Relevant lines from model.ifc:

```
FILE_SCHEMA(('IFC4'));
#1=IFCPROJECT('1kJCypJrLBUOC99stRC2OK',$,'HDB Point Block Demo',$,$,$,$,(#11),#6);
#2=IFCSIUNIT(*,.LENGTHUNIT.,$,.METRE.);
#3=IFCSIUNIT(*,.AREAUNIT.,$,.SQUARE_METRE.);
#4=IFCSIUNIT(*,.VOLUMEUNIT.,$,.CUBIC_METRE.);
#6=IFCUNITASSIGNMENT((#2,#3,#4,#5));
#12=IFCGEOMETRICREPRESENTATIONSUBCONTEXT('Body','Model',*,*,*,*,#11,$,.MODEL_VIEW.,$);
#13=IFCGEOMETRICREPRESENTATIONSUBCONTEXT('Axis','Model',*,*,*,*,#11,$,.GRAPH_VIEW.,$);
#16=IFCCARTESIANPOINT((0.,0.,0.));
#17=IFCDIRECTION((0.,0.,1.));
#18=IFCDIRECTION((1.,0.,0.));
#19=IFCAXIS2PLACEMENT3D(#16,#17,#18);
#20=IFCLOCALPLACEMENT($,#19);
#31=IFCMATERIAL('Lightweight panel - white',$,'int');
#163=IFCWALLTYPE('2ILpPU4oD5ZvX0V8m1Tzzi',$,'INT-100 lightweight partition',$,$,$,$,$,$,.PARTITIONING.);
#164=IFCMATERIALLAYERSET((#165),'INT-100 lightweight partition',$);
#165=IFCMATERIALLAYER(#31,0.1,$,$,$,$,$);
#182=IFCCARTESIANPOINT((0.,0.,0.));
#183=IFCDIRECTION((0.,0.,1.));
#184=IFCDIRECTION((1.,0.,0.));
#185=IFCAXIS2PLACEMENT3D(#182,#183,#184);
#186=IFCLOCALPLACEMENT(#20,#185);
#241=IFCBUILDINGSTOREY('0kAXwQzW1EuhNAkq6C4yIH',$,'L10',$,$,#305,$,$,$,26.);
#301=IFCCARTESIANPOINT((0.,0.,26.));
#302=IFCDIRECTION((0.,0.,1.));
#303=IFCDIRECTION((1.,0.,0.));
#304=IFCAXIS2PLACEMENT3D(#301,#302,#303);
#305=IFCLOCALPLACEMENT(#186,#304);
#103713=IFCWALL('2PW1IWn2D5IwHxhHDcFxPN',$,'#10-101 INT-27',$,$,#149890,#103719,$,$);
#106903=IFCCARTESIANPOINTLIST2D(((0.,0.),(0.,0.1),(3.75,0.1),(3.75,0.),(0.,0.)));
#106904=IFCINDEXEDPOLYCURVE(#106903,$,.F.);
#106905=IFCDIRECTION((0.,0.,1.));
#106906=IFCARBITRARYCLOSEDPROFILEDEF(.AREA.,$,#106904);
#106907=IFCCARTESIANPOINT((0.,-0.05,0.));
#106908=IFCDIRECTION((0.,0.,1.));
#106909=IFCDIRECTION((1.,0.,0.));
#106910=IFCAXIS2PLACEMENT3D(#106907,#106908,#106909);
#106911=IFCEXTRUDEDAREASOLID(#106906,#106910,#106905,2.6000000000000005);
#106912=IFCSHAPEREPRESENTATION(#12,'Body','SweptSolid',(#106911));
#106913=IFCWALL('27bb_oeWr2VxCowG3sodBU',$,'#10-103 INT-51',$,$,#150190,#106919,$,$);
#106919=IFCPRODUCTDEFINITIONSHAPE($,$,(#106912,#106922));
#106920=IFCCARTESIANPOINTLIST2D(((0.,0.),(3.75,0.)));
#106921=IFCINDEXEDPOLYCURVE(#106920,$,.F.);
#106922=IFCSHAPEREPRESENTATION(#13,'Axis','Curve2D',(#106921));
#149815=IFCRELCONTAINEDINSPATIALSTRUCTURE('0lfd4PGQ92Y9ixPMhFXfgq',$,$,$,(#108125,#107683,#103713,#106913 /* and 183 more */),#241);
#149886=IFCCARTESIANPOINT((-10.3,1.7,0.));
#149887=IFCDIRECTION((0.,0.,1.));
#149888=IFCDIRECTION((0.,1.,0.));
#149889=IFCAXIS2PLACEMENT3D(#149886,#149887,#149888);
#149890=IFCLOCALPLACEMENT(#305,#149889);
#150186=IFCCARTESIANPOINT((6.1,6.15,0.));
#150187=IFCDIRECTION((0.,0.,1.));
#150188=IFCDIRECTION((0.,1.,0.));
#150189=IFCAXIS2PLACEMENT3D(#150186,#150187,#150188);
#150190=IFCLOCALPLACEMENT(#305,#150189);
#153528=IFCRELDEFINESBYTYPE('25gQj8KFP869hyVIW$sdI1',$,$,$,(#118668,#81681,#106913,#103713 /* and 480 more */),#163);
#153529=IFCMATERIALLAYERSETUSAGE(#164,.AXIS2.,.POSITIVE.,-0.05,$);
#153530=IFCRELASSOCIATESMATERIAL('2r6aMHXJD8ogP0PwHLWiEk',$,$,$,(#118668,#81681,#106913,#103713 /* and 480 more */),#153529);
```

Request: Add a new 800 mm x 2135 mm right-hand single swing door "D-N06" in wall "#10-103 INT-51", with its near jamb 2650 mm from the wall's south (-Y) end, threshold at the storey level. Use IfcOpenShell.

```python
import numpy as np
import ifcopenshell
import ifcopenshell.api.feature
import ifcopenshell.api.geometry
import ifcopenshell.api.root
import ifcopenshell.api.spatial
import ifcopenshell.geom
import ifcopenshell.util.element
import ifcopenshell.util.placement
import ifcopenshell.util.representation
import ifcopenshell.util.shape
import ifcopenshell.util.unit

model = ifcopenshell.open("model.ifc")
unit_scale = ifcopenshell.util.unit.calculate_unit_scale(model)
settings = ifcopenshell.geom.settings()


def volume(element):
    """Net volume in cubic metres, openings subtracted."""
    shape = ifcopenshell.geom.create_shape(settings, element)
    return ifcopenshell.util.shape.get_volume(shape.geometry)


wall = model.by_id(106913)
storey = ifcopenshell.util.element.get_container(wall, ifc_class="IfcBuildingStorey")
context = ifcopenshell.util.representation.get_context(model, "Model", "Body", "MODEL_VIEW")
before = volume(wall)

width, height, from_end, sill = 0.8, 2.135, 2.65, 0.0  # metres

# The wall runs along its own X axis, and the end named is its -X end.
wall_shape = ifcopenshell.geom.create_shape(settings, wall)
x, y, z = ifcopenshell.util.shape.get_vertices(wall_shape.geometry).T
start = x.min() + from_end
face, thickness = float(y.min()), float(y.max() - y.min())
wall_matrix = ifcopenshell.util.placement.get_local_placement(wall.ObjectPlacement)
level = ifcopenshell.util.placement.get_local_placement(storey.ObjectPlacement)[2, 3]


def in_wall(x, y):
    """Placement at x, y metres in the wall's axes, at sill height."""
    matrix = wall_matrix.copy()
    matrix[:, 3] = wall_matrix @ np.array([x / unit_scale, y / unit_scale, 0.0, 1.0])
    matrix[2, 3] = level + sill / unit_scale
    return matrix


# Opening: a box that overshoots both wall faces by 50 mm.
opening = ifcopenshell.api.root.create_entity(model, ifc_class="IfcOpeningElement", predefined_type="OPENING")
box = ifcopenshell.api.geometry.add_wall_representation(
    model, context=context, length=width, height=height, thickness=thickness + 0.1
)
ifcopenshell.api.geometry.assign_representation(model, product=opening, representation=box)
ifcopenshell.api.geometry.edit_object_placement(model, product=opening, matrix=in_wall(start, face - 0.05), is_si=False)
ifcopenshell.api.feature.add_feature(model, feature=opening, element=wall)

door = ifcopenshell.api.root.create_entity(model, ifc_class="IfcDoor", name="D-N06", predefined_type="DOOR")
door.OverallWidth, door.OverallHeight = width / unit_scale, height / unit_scale
door.OperationType = "SINGLE_SWING_RIGHT"
body = ifcopenshell.api.geometry.add_door_representation(
    model,
    context=context,
    overall_width=door.OverallWidth,
    overall_height=door.OverallHeight,
    operation_type="SINGLE_SWING_RIGHT",
    lining_properties={"LiningDepth": thickness / unit_scale, "ThresholdDepth": thickness / unit_scale},
)
ifcopenshell.api.geometry.assign_representation(model, product=door, representation=body)
ifcopenshell.api.spatial.assign_container(model, products=[door], relating_structure=storey)
ifcopenshell.api.feature.add_filling(model, opening=opening, element=door)

# The lining spans the wall, so the door starts at the wall face.
ifcopenshell.api.geometry.edit_object_placement(model, product=door, matrix=in_wall(start, face), is_si=False)

after = volume(wall)

print(f"wall volume {before:.3f} -> {after:.3f} m3")

model.write("model_v2.ifc")
```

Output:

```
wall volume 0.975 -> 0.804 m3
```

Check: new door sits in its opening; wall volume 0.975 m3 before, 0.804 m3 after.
